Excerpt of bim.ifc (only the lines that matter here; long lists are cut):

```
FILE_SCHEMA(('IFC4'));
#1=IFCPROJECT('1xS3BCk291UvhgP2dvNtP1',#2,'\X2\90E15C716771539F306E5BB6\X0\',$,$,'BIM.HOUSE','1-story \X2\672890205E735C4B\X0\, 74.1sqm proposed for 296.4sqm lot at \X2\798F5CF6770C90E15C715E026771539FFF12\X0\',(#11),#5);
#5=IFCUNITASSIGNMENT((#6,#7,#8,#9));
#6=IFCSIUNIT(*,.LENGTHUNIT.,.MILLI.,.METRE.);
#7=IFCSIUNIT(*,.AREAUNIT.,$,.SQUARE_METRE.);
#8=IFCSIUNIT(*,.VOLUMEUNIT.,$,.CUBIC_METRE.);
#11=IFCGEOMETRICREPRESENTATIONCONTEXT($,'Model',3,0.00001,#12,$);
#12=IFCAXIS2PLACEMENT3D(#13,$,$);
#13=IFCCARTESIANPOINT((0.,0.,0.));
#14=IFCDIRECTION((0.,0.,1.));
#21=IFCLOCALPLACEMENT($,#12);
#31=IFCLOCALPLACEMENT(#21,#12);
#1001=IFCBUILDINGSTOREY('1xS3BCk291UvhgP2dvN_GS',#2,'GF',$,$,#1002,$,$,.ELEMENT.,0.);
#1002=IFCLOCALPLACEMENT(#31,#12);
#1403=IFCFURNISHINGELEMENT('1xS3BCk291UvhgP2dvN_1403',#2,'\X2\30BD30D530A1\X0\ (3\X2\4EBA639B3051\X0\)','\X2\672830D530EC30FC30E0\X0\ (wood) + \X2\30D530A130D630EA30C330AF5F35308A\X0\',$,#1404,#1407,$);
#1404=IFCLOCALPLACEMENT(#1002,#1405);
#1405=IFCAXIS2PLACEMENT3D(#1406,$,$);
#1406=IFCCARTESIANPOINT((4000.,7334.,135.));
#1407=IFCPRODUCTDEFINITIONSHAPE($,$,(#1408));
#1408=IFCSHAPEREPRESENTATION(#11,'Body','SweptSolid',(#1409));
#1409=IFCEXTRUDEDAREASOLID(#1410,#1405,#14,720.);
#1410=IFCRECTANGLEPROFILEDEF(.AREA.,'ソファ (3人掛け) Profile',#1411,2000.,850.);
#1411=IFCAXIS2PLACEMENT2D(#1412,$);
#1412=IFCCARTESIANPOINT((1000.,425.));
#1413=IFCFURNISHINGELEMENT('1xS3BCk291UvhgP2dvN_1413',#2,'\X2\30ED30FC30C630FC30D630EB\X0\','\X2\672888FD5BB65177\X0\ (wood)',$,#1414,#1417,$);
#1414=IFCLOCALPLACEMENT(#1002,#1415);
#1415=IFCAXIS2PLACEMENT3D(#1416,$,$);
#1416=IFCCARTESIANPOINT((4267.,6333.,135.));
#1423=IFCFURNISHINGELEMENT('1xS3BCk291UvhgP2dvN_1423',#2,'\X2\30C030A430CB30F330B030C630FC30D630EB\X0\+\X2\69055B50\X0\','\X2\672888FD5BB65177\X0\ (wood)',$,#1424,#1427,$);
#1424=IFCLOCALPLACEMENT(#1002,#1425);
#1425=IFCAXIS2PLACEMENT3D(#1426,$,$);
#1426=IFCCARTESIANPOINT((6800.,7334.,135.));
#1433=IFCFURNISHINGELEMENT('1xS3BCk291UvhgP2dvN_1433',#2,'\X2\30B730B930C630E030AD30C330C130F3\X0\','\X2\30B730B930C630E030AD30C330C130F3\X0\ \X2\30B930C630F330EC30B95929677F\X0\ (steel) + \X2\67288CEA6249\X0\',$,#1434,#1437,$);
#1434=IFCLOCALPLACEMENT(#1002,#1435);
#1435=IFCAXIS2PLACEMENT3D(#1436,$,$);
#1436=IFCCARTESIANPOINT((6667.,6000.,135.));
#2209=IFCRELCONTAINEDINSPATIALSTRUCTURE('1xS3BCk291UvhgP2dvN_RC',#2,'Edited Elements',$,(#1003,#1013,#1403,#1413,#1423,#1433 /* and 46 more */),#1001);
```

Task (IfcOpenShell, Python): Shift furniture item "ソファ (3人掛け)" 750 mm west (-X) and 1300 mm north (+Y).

```python
import ifcopenshell
import ifcopenshell.api.geometry
import ifcopenshell.util.placement
import ifcopenshell.util.unit

model = ifcopenshell.open("bim.ifc")
unit_scale = ifcopenshell.util.unit.calculate_unit_scale(model)

item = model.by_id(1403)
matrix = ifcopenshell.util.placement.get_local_placement(item.ObjectPlacement)
matrix[0, 3] -= 0.75 / unit_scale
matrix[1, 3] += 1.3 / unit_scale
ifcopenshell.api.geometry.edit_object_placement(model, product=item, matrix=matrix, is_si=False)

print(ifcopenshell.util.placement.get_local_placement(item.ObjectPlacement).round(3) + 0.0)

model.write("bim_v2.ifc")
```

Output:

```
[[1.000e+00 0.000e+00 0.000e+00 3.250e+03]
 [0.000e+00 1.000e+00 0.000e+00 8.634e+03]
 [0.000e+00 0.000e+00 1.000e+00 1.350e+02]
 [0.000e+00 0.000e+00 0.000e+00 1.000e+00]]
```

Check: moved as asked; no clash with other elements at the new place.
